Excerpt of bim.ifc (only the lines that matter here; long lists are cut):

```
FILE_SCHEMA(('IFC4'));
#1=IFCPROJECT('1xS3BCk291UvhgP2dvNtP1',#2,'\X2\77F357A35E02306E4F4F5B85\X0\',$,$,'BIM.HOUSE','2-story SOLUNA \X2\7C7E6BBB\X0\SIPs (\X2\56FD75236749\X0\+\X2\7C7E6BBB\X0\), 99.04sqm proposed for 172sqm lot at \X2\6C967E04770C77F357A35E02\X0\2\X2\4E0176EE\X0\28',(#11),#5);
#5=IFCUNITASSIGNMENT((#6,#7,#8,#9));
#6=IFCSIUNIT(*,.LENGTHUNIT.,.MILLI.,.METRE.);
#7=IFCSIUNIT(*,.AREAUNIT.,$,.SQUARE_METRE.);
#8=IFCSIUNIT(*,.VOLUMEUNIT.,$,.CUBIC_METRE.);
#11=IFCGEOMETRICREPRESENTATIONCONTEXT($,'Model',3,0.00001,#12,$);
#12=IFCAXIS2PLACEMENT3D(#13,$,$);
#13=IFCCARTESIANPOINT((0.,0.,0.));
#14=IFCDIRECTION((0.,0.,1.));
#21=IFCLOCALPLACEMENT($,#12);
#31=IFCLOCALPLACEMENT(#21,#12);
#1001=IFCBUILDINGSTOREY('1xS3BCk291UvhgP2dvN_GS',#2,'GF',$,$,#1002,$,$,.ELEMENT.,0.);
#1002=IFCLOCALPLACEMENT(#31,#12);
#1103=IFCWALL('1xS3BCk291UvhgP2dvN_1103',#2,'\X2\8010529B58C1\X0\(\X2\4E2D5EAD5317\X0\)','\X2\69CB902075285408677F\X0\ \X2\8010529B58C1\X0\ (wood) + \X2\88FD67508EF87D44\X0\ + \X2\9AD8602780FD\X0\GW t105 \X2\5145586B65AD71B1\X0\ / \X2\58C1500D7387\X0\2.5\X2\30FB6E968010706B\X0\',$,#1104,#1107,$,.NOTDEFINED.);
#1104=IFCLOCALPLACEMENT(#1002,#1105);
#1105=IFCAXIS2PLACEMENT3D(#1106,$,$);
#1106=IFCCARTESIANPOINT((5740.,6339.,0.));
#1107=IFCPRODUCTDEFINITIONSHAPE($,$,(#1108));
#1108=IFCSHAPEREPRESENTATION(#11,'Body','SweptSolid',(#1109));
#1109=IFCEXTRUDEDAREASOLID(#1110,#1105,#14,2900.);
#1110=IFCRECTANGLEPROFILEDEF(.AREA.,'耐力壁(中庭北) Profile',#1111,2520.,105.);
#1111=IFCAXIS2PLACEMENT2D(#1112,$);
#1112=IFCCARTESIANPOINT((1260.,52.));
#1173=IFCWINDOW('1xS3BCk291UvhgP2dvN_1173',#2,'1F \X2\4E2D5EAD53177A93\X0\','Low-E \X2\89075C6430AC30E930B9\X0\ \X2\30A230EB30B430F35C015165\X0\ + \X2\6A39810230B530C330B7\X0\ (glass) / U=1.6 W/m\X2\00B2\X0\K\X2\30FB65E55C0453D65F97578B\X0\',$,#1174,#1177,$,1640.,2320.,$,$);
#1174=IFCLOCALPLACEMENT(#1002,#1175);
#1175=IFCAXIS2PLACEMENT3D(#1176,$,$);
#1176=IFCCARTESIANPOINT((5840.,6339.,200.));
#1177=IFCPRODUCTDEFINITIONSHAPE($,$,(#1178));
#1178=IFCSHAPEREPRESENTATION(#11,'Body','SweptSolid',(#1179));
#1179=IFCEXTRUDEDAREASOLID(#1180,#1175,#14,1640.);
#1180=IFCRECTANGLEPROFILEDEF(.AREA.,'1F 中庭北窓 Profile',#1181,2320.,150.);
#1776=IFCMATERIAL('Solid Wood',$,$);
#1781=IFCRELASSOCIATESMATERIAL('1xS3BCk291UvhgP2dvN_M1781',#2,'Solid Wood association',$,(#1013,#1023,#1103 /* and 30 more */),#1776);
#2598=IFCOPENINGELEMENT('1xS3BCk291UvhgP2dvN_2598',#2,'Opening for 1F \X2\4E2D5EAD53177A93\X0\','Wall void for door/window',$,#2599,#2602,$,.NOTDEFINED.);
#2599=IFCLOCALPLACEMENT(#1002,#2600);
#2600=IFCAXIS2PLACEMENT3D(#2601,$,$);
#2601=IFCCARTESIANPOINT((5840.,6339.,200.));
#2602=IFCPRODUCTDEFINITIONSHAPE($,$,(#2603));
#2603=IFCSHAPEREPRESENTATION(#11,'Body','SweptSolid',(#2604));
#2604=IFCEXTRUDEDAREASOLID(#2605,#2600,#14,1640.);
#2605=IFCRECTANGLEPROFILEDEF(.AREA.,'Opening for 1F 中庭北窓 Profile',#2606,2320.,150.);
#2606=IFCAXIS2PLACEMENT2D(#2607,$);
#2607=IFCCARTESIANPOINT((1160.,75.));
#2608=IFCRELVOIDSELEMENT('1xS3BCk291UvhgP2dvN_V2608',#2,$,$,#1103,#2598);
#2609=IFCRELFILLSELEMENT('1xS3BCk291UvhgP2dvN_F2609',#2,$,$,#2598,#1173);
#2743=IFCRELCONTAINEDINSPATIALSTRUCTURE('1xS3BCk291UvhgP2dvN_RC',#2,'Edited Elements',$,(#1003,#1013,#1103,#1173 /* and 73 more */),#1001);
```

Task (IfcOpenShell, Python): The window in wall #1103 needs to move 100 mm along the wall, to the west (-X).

```python
import ifcopenshell
import ifcopenshell.api.geometry
import ifcopenshell.util.placement

model = ifcopenshell.open("bim.ifc")

window = model.by_id(1173)
opening = window.FillsVoids[0].RelatingOpeningElement
wall = opening.VoidsElements[0].RelatingBuildingElement

wall_matrix = ifcopenshell.util.placement.get_local_placement(wall.ObjectPlacement)
shift = wall_matrix[:3, 0] * -100.0
before = ifcopenshell.util.placement.get_local_placement(window.ObjectPlacement)[:3, 3].copy()

# The window is not placed relative to its opening, so move both.
for product in (opening, window):
    matrix = ifcopenshell.util.placement.get_local_placement(product.ObjectPlacement)
    matrix[:3, 3] += shift
    ifcopenshell.api.geometry.edit_object_placement(model, product=product, matrix=matrix, is_si=False)

after = ifcopenshell.util.placement.get_local_placement(window.ObjectPlacement)[:3, 3]
print("window moved by", (after - before).round(3) + 0.0)

model.write("bim_rev.ifc")
```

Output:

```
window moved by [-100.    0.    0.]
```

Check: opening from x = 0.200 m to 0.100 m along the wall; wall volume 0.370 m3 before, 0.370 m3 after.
